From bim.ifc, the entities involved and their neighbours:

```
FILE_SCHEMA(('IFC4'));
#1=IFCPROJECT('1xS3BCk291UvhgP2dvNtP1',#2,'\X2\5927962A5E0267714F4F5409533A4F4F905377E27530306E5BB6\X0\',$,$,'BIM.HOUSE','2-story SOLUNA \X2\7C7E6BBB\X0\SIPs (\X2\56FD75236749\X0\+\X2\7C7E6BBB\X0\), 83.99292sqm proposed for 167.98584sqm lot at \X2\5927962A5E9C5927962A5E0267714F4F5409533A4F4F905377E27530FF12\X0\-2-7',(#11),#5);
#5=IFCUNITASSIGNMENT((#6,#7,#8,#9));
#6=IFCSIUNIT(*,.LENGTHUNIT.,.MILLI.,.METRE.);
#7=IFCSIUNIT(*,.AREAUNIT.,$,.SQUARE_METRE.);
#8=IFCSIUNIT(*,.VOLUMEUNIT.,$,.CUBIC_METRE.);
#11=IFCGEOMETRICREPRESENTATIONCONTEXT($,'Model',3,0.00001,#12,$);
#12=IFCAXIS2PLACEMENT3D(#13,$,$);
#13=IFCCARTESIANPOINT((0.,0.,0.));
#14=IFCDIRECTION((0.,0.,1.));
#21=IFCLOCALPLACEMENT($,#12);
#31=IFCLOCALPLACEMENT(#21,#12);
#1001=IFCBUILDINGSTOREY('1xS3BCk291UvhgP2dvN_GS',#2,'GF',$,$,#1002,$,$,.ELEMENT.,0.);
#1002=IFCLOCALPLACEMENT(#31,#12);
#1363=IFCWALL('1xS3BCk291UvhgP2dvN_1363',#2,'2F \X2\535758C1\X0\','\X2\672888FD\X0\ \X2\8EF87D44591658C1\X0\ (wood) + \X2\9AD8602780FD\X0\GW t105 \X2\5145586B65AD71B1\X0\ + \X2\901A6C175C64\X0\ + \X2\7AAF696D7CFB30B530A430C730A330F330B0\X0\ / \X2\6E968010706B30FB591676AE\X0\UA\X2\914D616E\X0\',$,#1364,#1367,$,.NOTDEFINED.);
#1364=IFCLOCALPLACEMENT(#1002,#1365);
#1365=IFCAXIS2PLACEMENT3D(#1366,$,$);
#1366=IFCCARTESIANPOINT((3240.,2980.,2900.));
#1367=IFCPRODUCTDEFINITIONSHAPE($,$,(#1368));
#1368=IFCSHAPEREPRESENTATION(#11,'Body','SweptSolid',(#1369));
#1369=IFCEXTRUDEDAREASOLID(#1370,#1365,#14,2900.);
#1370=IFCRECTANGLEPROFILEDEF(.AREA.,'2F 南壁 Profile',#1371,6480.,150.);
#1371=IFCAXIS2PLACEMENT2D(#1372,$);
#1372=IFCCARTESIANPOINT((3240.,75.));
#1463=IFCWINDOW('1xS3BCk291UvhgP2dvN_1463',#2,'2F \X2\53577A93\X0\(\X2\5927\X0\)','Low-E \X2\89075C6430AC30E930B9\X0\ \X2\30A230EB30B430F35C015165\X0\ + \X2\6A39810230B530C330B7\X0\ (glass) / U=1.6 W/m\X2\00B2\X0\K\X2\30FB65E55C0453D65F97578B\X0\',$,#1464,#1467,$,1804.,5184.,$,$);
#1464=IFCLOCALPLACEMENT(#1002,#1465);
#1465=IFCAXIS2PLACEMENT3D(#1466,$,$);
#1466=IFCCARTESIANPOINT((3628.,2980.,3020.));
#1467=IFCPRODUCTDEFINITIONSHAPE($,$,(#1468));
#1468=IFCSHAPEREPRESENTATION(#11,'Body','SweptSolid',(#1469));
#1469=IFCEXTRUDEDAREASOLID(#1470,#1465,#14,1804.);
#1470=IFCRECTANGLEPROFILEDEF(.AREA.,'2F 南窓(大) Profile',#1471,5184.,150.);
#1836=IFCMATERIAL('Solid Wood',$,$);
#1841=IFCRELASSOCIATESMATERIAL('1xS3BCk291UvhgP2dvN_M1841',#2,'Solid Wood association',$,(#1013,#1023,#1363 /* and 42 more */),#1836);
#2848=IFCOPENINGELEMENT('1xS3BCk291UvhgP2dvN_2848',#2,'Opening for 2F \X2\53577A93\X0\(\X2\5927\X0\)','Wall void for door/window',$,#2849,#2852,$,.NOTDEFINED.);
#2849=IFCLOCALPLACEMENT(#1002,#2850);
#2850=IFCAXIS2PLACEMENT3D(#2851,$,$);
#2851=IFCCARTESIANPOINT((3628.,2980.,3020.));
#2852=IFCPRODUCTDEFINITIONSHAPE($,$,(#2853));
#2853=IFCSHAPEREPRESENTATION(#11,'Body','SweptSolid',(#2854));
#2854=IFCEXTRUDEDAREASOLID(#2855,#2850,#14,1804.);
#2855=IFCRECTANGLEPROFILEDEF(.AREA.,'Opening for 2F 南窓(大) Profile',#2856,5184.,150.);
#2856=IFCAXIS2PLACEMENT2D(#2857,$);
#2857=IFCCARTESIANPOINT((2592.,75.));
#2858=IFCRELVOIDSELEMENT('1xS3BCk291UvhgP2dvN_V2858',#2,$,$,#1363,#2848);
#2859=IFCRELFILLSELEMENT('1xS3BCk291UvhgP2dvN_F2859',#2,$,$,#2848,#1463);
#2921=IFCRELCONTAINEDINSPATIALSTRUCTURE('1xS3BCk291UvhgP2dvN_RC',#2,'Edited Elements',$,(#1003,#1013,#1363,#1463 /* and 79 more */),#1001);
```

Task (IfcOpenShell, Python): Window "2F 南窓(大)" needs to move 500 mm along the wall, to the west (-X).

```python
import ifcopenshell
import ifcopenshell.api.geometry
import ifcopenshell.util.placement
import ifcopenshell.util.unit

model = ifcopenshell.open("bim.ifc")
unit_scale = ifcopenshell.util.unit.calculate_unit_scale(model)

window = model.by_guid("1xS3BCk291UvhgP2dvN_1463")
opening = window.FillsVoids[0].RelatingOpeningElement
wall = opening.VoidsElements[0].RelatingBuildingElement

wall_matrix = ifcopenshell.util.placement.get_local_placement(wall.ObjectPlacement)
shift = wall_matrix[:3, 0] * -0.5 / unit_scale
before = ifcopenshell.util.placement.get_local_placement(window.ObjectPlacement)[:3, 3].copy()

# The window is not placed relative to its opening, so move both.
for product in (opening, window):
    matrix = ifcopenshell.util.placement.get_local_placement(product.ObjectPlacement)
    matrix[:3, 3] += shift
    ifcopenshell.api.geometry.edit_object_placement(model, product=product, matrix=matrix, is_si=False)

after = ifcopenshell.util.placement.get_local_placement(window.ObjectPlacement)[:3, 3]
print("window moved by", (after - before).round(3) + 0.0)

model.write("bim_updated.ifc")
```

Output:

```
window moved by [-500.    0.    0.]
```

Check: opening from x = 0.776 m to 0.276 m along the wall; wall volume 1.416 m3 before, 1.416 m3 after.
